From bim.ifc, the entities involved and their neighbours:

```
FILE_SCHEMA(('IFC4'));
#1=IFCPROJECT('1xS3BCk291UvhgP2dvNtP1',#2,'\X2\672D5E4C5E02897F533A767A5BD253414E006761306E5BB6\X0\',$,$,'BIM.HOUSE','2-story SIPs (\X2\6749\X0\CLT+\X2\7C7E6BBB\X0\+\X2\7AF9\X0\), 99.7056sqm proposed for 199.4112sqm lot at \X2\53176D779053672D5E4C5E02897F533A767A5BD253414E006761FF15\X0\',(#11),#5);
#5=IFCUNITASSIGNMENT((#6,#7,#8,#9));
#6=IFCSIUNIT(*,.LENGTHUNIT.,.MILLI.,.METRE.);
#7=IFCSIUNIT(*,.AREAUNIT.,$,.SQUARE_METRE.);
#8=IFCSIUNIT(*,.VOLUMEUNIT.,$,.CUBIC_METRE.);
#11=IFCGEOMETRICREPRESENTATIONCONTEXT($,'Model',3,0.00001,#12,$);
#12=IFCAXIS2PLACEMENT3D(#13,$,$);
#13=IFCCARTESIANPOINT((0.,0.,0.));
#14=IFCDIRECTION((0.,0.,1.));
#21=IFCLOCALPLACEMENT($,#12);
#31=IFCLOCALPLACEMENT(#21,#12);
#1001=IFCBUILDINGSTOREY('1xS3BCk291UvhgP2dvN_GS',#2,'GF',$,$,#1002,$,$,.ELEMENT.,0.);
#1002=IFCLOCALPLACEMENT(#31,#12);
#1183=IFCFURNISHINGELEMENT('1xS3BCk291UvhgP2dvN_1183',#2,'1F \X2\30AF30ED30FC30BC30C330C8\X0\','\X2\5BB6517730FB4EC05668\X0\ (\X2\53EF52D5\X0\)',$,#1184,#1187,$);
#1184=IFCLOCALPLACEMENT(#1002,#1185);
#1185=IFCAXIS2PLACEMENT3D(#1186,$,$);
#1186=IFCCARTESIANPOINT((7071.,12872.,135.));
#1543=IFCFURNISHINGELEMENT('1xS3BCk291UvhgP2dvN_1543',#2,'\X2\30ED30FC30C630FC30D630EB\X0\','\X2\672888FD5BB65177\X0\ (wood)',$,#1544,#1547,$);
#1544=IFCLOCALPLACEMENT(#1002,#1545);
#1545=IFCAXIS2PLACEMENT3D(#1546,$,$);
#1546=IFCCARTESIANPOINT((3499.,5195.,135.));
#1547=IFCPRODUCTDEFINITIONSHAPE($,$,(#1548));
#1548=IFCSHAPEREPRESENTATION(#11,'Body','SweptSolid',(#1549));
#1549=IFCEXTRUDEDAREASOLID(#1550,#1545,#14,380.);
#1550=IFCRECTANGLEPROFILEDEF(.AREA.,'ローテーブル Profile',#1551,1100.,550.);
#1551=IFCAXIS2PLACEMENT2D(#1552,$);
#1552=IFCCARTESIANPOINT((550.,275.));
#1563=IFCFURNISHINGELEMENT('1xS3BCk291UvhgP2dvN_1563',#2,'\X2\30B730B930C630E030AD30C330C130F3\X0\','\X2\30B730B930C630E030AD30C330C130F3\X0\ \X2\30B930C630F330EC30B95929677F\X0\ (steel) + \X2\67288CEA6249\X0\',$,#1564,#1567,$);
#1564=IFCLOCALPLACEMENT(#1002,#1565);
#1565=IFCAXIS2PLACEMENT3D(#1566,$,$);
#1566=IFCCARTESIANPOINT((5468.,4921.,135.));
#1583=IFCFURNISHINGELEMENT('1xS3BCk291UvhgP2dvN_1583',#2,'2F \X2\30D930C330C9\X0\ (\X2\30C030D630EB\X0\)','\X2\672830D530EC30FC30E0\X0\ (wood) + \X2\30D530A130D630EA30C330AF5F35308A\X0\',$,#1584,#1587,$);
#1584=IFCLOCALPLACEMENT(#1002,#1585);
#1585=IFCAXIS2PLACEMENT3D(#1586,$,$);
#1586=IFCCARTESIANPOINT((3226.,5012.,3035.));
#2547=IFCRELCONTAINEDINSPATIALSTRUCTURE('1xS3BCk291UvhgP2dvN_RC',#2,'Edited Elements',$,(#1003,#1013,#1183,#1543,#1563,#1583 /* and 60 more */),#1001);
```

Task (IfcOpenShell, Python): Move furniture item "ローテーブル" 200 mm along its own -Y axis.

```python
import ifcopenshell
import ifcopenshell.api.geometry
import ifcopenshell.util.placement
import ifcopenshell.util.unit

model = ifcopenshell.open("bim.ifc")
unit_scale = ifcopenshell.util.unit.calculate_unit_scale(model)

item = model.by_guid("1xS3BCk291UvhgP2dvN_1543")
matrix = ifcopenshell.util.placement.get_local_placement(item.ObjectPlacement)
matrix[:3, 3] -= matrix[:3, 1] * 0.2 / unit_scale
ifcopenshell.api.geometry.edit_object_placement(model, product=item, matrix=matrix, is_si=False)

print(ifcopenshell.util.placement.get_local_placement(item.ObjectPlacement).round(3) + 0.0)

model.write("bim_edited.ifc")
```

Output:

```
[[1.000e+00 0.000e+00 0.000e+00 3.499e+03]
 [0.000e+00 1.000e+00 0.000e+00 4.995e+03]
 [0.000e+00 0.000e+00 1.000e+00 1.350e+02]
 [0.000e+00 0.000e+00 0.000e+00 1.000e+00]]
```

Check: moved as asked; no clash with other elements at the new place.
